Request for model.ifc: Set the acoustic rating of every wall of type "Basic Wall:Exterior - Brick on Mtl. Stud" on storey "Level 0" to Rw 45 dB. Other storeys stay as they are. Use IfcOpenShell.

First a look at what the model holds.

```python
import ifcopenshell
import ifcopenshell.util.element

model = ifcopenshell.open("model.ifc")
print(model.schema)
storey = next(s for s in model.by_type("IfcBuildingStorey") if s.Name == "Level 0")
walls = [e for e in ifcopenshell.util.element.get_decomposition(storey) if e.is_a("IfcWall")]
seen = {}
for e in walls:
    element_type = ifcopenshell.util.element.get_type(e)
    key = (element_type.Name if element_type != e and element_type else None, ifcopenshell.util.element.get_pset(e, "Pset_WallCommon", "AcousticRating"))
    seen[key] = seen.get(key, 0) + 1
for (name, value), count in sorted(seen.items(), key=str):
    print(count, "x", name, "|", value)
```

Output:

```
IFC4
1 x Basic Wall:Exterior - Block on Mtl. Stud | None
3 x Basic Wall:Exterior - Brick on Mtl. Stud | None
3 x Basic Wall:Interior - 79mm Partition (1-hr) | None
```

```python
import ifcopenshell
import ifcopenshell.api.pset
import ifcopenshell.util.element

model = ifcopenshell.open("model.ifc")

storey = next(s for s in model.by_type("IfcBuildingStorey") if s.Name == "Level 0")
walls = [e for e in ifcopenshell.util.element.get_decomposition(storey) if e.is_a("IfcWall")]

count = 0
for e in walls:
    element_type = ifcopenshell.util.element.get_type(e)
    if element_type in (None, e) or element_type.Name != "Basic Wall:Exterior - Brick on Mtl. Stud":
        continue
    # add_pset returns the element's existing set when there is one.
    pset = ifcopenshell.api.pset.add_pset(model, product=e, name="Pset_WallCommon")
    ifcopenshell.api.pset.edit_pset(model, pset=pset, properties={"AcousticRating": "Rw 45 dB"})
    count += 1

print(count, "walls updated")

model.write("model_v2.ifc")
```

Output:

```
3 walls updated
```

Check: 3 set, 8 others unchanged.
